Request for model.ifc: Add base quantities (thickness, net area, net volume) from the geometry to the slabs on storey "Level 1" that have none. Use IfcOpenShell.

First a look at what the model holds.

```python
import ifcopenshell
import ifcopenshell.util.element
import ifcopenshell.util.unit

model = ifcopenshell.open("model.ifc")
print(model.schema)
for unit_type in ("LENGTHUNIT", "AREAUNIT", "VOLUMEUNIT"):
    print(unit_type, ifcopenshell.util.unit.calculate_unit_scale(model, unit_type))
storey = next(s for s in model.by_type("IfcBuildingStorey") if s.Name == "Level 1")
slabs = [e for e in ifcopenshell.util.element.get_decomposition(storey) if e.is_a("IfcSlab")]
for e in sorted(slabs, key=lambda e: e.id()):
    print(e.id(), e.is_a(), e.Name, list(ifcopenshell.util.element.get_psets(e, qtos_only=True)), sep=" | ")
```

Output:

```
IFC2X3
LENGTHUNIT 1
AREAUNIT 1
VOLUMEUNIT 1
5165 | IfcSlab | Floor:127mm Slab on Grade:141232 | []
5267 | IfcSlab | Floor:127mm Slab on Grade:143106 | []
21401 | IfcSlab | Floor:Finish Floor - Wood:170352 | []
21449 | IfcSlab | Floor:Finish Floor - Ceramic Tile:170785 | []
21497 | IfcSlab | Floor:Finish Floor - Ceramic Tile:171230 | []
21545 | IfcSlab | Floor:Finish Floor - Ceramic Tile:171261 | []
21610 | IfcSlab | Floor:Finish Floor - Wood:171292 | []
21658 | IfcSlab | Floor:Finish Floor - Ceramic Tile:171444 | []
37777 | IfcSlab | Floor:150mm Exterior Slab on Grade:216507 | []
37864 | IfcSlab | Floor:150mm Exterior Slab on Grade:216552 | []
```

```python
import ifcopenshell
import ifcopenshell.api.pset
import ifcopenshell.geom
import ifcopenshell.util.element
import ifcopenshell.util.shape
import ifcopenshell.util.unit

model = ifcopenshell.open("model.ifc")
unit_scale = ifcopenshell.util.unit.calculate_unit_scale(model)
area_scale = ifcopenshell.util.unit.calculate_unit_scale(model, "AREAUNIT")
volume_scale = ifcopenshell.util.unit.calculate_unit_scale(model, "VOLUMEUNIT")
settings = ifcopenshell.geom.settings()

storey = next(s for s in model.by_type("IfcBuildingStorey") if s.Name == "Level 1")
slabs = [e for e in ifcopenshell.util.element.get_decomposition(storey) if e.is_a("IfcSlab")]

for e in sorted(slabs, key=lambda e: e.id()):
    if ifcopenshell.util.element.get_psets(e, qtos_only=True, should_inherit=False):
        continue
    # Geometry comes back in metres, in the element's own axes.
    shape = ifcopenshell.geom.create_shape(settings, e)
    values = {
        "Width": ifcopenshell.util.shape.get_z(shape.geometry) / unit_scale,
        "NetArea": ifcopenshell.util.shape.get_footprint_area(shape.geometry) / area_scale,
        "NetVolume": ifcopenshell.util.shape.get_volume(shape.geometry) / volume_scale,
    }
    qto = ifcopenshell.api.pset.add_qto(model, product=e, name="BaseQuantities")
    ifcopenshell.api.pset.edit_qto(model, qto=qto, properties=values)
    print(e.id(), {k: round(v, 3) for k, v in values.items()})

model.write("model_updated.ifc")
```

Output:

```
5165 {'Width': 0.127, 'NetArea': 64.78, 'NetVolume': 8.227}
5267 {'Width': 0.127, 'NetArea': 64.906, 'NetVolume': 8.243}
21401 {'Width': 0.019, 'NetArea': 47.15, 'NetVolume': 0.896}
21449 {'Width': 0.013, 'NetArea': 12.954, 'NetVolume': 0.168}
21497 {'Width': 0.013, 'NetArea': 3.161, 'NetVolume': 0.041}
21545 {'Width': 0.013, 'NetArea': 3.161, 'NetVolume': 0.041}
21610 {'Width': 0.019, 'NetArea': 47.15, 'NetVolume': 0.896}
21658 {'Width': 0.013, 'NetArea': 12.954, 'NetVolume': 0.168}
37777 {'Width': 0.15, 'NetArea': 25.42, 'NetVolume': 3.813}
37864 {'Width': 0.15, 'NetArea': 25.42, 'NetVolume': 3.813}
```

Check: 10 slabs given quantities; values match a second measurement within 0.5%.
